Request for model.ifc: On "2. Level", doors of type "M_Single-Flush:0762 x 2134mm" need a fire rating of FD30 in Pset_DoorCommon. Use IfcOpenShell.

First a look at what the model holds.

```python
import ifcopenshell
import ifcopenshell.util.element

model = ifcopenshell.open("model.ifc")
print(model.schema)
storey = next(s for s in model.by_type("IfcBuildingStorey") if s.Name == "2. Level")
doors = [e for e in ifcopenshell.util.element.get_decomposition(storey) if e.is_a("IfcDoor")]
seen = {}
for e in doors:
    element_type = ifcopenshell.util.element.get_type(e)
    key = (element_type.Name if element_type != e and element_type else None, ifcopenshell.util.element.get_pset(e, "Pset_DoorCommon", "FireRating"))
    seen[key] = seen.get(key, 0) + 1
for (name, value), count in sorted(seen.items(), key=str):
    print(count, "x", name, "|", value)
```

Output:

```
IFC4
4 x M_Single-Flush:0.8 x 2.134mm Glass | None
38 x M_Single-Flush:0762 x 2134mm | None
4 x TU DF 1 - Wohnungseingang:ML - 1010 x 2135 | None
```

```python
import ifcopenshell
import ifcopenshell.api.pset
import ifcopenshell.util.element

model = ifcopenshell.open("model.ifc")

storey = next(s for s in model.by_type("IfcBuildingStorey") if s.Name == "2. Level")
doors = [e for e in ifcopenshell.util.element.get_decomposition(storey) if e.is_a("IfcDoor")]

count = 0
for e in doors:
    element_type = ifcopenshell.util.element.get_type(e)
    if element_type in (None, e) or element_type.Name != "M_Single-Flush:0762 x 2134mm":
        continue
    # add_pset returns the element's existing set when there is one.
    pset = ifcopenshell.api.pset.add_pset(model, product=e, name="Pset_DoorCommon")
    ifcopenshell.api.pset.edit_pset(model, pset=pset, properties={"FireRating": "FD30"})
    count += 1

print(count, "doors updated")

model.write("model_edited.ifc")
```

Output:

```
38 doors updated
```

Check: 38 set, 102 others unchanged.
